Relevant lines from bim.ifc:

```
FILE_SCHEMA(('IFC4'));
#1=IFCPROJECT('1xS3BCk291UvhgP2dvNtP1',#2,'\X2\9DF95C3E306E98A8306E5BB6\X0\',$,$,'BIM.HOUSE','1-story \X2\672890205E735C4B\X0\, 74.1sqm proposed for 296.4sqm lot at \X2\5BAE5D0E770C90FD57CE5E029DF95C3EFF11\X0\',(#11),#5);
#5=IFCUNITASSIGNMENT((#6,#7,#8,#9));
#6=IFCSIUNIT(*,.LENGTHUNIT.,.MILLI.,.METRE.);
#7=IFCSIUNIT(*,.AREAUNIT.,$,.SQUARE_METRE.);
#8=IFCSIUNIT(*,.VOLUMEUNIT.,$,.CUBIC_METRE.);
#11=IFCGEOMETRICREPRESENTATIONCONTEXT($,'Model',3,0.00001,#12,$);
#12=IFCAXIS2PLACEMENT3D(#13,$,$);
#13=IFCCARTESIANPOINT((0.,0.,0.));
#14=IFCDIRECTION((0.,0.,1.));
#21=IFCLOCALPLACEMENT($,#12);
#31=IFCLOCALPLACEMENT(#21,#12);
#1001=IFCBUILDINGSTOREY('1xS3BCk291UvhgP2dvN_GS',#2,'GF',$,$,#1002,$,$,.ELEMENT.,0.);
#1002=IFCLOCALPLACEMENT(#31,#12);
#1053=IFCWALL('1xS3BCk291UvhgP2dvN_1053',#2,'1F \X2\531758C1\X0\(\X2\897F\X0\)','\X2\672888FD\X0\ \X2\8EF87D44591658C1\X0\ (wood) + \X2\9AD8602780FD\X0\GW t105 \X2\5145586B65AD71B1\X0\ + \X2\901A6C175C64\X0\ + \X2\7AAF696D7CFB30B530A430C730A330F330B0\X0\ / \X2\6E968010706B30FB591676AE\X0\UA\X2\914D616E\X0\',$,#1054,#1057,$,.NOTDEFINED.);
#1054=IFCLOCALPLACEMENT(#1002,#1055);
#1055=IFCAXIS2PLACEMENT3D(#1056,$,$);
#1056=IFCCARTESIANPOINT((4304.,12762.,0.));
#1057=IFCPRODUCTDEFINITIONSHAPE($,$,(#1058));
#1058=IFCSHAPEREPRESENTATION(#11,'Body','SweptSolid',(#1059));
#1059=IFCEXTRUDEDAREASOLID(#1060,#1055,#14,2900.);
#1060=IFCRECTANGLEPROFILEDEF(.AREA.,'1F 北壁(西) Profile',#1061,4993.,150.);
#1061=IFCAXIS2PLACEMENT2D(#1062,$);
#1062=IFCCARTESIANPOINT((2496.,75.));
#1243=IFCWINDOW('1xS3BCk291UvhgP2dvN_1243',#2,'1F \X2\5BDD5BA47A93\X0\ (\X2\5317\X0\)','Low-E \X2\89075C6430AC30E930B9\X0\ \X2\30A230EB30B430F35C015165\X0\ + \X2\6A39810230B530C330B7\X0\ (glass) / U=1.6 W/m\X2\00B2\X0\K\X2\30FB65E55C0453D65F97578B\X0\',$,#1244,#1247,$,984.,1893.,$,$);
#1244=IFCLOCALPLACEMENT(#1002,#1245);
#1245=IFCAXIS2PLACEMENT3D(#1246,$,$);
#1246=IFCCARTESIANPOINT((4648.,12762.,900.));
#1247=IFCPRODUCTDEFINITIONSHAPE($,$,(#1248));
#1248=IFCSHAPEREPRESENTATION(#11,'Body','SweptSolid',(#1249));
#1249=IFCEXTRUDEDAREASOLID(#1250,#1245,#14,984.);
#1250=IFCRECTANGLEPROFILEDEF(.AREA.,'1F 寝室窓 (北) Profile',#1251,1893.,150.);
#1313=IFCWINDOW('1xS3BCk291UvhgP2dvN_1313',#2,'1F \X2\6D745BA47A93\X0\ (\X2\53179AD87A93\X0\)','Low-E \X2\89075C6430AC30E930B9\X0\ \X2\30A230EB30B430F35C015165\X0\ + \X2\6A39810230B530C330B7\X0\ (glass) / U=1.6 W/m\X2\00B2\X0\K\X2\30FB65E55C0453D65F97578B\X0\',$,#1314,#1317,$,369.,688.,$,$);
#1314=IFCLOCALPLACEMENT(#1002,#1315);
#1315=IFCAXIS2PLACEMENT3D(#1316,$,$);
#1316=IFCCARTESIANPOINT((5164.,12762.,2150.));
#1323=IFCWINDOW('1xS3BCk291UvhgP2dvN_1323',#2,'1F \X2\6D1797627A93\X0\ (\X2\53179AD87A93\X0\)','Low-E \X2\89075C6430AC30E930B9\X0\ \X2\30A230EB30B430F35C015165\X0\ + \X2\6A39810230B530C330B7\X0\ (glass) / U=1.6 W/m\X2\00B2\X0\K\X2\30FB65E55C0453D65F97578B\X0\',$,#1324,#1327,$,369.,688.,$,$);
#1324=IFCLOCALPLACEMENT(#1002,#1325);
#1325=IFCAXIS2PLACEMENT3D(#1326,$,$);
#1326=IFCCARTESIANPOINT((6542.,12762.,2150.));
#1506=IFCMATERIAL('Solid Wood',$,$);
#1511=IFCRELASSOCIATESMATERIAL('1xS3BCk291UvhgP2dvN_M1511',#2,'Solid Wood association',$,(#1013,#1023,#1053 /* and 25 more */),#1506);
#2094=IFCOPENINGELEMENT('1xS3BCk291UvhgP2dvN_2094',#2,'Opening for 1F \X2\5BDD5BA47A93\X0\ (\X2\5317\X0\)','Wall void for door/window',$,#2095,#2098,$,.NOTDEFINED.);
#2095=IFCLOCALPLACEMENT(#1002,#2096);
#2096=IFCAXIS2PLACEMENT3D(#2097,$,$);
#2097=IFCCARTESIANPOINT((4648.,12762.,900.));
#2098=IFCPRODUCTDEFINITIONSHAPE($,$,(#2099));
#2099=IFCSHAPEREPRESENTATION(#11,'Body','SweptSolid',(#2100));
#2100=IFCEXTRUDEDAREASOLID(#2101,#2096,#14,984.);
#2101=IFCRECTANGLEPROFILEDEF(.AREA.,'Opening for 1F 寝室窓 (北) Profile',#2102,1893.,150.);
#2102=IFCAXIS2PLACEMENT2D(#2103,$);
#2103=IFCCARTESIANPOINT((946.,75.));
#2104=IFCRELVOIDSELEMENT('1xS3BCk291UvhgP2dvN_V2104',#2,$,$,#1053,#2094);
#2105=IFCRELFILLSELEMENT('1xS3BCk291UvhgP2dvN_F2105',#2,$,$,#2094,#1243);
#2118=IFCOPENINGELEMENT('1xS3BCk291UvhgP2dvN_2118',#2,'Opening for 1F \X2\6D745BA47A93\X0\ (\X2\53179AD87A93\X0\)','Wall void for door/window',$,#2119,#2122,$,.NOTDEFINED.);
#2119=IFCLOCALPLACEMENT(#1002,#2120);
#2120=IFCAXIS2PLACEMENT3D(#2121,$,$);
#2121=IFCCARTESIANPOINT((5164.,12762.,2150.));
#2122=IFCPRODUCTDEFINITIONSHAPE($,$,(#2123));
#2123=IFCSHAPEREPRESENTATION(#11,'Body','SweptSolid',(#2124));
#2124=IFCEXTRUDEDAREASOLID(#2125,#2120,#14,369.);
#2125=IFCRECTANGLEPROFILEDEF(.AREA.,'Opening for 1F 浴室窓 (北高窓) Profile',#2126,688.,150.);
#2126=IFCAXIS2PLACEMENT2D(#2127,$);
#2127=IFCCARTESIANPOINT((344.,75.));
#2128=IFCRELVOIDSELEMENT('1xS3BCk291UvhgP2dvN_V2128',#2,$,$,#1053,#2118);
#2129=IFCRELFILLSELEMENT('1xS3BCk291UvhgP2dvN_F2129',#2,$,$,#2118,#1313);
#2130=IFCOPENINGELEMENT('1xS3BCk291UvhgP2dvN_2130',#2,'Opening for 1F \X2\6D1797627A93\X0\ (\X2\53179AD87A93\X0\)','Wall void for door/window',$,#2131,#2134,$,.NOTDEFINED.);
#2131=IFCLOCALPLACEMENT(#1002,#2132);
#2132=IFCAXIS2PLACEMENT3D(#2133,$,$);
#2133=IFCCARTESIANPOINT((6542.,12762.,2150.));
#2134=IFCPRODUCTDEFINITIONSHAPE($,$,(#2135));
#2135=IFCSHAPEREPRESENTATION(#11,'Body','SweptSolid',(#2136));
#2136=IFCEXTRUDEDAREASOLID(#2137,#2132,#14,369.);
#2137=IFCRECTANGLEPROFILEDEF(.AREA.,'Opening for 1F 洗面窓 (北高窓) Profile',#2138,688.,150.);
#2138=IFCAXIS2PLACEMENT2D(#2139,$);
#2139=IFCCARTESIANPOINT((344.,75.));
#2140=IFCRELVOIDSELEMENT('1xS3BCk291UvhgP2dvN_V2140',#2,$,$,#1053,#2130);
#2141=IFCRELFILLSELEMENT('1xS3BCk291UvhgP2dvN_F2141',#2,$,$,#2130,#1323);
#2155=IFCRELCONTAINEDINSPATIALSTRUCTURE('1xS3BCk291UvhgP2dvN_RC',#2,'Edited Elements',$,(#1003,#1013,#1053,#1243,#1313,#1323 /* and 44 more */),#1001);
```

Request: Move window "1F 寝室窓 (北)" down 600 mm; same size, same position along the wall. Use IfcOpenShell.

```python
import numpy as np
import ifcopenshell
import ifcopenshell.api.geometry
import ifcopenshell.util.placement
import ifcopenshell.util.unit

model = ifcopenshell.open("bim.ifc")
unit_scale = ifcopenshell.util.unit.calculate_unit_scale(model)

window = model.by_guid("1xS3BCk291UvhgP2dvN_1243")
opening = window.FillsVoids[0].RelatingOpeningElement
dz = -600.0

shift = np.array([0.0, 0.0, dz])
# The window is not placed relative to its opening, so move both.
for product in (opening, window):
    matrix = ifcopenshell.util.placement.get_local_placement(product.ObjectPlacement)
    matrix[:3, 3] += shift
    ifcopenshell.api.geometry.edit_object_placement(model, product=product, matrix=matrix, is_si=False)

print(f"moved by {dz * unit_scale:+.3f} m")

model.write("bim_updated.ifc")
```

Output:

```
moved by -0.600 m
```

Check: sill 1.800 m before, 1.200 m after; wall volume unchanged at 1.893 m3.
